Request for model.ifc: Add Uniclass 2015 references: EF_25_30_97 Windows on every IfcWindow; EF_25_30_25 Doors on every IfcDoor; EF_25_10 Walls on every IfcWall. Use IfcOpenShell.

First a look at what the model holds.

```python
import ifcopenshell

model = ifcopenshell.open("model.ifc")
print(model.schema)
print("classifications:", [c.Name for c in model.by_type("IfcClassification")])
for ifc_class in ("IfcDoor", "IfcRoof", "IfcStair", "IfcWall", "IfcWindow"):
    print(ifc_class, len(model.by_type(ifc_class)))
```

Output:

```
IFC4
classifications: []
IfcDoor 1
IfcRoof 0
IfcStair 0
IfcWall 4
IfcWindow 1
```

```python
import ifcopenshell
import ifcopenshell.api.classification

model = ifcopenshell.open("model.ifc")

system = ifcopenshell.api.classification.add_classification(model, classification="Uniclass 2015")

codes = {
    "IfcWindow": ("EF_25_30_97", "Windows"),
    "IfcDoor": ("EF_25_30_25", "Doors"),
    "IfcWall": ("EF_25_10", "Walls"),
}
for ifc_class, (code, name) in codes.items():
    products = model.by_type(ifc_class)
    ifcopenshell.api.classification.add_reference(
        model, products=products, classification=system, identification=code, name=name
    )
    print(code, len(products))

model.write("model-out.ifc")
```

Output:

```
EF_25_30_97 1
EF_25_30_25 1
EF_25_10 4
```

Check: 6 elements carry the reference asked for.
